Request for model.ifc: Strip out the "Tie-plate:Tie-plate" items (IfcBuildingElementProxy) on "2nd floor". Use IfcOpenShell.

First a look at what the model holds.

```python
import ifcopenshell
import ifcopenshell.util.element

model = ifcopenshell.open("model.ifc")
print(model.schema)
storey = next(s for s in model.by_type("IfcBuildingStorey") if s.Name == "2nd floor")
proxies = [e for e in ifcopenshell.util.element.get_decomposition(storey) if e.is_a("IfcBuildingElementProxy")]
seen = {}
for e in proxies:
    element_type = ifcopenshell.util.element.get_type(e)
    name = element_type.Name if element_type not in (None, e) else None
    seen[name] = seen.get(name, 0) + 1
for name, count in sorted(seen.items(), key=str):
    print(count, "x", name)
```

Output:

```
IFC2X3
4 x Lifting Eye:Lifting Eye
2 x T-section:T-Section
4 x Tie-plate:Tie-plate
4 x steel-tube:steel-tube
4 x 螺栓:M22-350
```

```python
import ifcopenshell
import ifcopenshell.api.root
import ifcopenshell.util.element

model = ifcopenshell.open("model.ifc")

storey = next(s for s in model.by_type("IfcBuildingStorey") if s.Name == "2nd floor")
proxies = [e for e in ifcopenshell.util.element.get_decomposition(storey) if e.is_a("IfcBuildingElementProxy")]
targets = [e for e in proxies if (t := ifcopenshell.util.element.get_type(e)) not in (None, e) and t.Name == "Tie-plate:Tie-plate"]

for e in targets:
    ifcopenshell.api.root.remove_product(model, product=e)
print(len(targets), "removed")

model.write("model_v2.ifc")
```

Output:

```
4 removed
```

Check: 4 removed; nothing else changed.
